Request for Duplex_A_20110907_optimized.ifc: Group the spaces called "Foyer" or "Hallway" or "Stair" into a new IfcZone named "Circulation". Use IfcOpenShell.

First a look at what the model holds.

```python
import ifcopenshell

model = ifcopenshell.open("Duplex_A_20110907_optimized.ifc")
print(model.schema)
seen = {}
for space in model.by_type("IfcSpace"):
    seen[space.LongName] = seen.get(space.LongName, 0) + 1
for name, count in sorted(seen.items(), key=str):
    print(count, "x", name)
print("zones:", [z.Name for z in model.by_type("IfcZone")][:20])
```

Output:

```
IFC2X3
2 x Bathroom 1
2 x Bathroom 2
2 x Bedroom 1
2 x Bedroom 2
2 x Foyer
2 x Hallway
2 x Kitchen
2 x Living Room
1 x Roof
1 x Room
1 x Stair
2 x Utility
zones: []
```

```python
import ifcopenshell
import ifcopenshell.api.group
import ifcopenshell.api.root

model = ifcopenshell.open("Duplex_A_20110907_optimized.ifc")

names = {"Foyer", "Hallway", "Stair"}
spaces = [s for s in model.by_type("IfcSpace") if s.LongName in names]

zone = ifcopenshell.api.root.create_entity(model, ifc_class="IfcZone", name="Circulation")
ifcopenshell.api.group.assign_group(model, products=spaces, group=zone)
print(len(spaces), "spaces in", zone.Name)

model.write("Duplex_A_20110907_optimized_v2.ifc")
```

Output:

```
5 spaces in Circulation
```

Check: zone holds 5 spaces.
